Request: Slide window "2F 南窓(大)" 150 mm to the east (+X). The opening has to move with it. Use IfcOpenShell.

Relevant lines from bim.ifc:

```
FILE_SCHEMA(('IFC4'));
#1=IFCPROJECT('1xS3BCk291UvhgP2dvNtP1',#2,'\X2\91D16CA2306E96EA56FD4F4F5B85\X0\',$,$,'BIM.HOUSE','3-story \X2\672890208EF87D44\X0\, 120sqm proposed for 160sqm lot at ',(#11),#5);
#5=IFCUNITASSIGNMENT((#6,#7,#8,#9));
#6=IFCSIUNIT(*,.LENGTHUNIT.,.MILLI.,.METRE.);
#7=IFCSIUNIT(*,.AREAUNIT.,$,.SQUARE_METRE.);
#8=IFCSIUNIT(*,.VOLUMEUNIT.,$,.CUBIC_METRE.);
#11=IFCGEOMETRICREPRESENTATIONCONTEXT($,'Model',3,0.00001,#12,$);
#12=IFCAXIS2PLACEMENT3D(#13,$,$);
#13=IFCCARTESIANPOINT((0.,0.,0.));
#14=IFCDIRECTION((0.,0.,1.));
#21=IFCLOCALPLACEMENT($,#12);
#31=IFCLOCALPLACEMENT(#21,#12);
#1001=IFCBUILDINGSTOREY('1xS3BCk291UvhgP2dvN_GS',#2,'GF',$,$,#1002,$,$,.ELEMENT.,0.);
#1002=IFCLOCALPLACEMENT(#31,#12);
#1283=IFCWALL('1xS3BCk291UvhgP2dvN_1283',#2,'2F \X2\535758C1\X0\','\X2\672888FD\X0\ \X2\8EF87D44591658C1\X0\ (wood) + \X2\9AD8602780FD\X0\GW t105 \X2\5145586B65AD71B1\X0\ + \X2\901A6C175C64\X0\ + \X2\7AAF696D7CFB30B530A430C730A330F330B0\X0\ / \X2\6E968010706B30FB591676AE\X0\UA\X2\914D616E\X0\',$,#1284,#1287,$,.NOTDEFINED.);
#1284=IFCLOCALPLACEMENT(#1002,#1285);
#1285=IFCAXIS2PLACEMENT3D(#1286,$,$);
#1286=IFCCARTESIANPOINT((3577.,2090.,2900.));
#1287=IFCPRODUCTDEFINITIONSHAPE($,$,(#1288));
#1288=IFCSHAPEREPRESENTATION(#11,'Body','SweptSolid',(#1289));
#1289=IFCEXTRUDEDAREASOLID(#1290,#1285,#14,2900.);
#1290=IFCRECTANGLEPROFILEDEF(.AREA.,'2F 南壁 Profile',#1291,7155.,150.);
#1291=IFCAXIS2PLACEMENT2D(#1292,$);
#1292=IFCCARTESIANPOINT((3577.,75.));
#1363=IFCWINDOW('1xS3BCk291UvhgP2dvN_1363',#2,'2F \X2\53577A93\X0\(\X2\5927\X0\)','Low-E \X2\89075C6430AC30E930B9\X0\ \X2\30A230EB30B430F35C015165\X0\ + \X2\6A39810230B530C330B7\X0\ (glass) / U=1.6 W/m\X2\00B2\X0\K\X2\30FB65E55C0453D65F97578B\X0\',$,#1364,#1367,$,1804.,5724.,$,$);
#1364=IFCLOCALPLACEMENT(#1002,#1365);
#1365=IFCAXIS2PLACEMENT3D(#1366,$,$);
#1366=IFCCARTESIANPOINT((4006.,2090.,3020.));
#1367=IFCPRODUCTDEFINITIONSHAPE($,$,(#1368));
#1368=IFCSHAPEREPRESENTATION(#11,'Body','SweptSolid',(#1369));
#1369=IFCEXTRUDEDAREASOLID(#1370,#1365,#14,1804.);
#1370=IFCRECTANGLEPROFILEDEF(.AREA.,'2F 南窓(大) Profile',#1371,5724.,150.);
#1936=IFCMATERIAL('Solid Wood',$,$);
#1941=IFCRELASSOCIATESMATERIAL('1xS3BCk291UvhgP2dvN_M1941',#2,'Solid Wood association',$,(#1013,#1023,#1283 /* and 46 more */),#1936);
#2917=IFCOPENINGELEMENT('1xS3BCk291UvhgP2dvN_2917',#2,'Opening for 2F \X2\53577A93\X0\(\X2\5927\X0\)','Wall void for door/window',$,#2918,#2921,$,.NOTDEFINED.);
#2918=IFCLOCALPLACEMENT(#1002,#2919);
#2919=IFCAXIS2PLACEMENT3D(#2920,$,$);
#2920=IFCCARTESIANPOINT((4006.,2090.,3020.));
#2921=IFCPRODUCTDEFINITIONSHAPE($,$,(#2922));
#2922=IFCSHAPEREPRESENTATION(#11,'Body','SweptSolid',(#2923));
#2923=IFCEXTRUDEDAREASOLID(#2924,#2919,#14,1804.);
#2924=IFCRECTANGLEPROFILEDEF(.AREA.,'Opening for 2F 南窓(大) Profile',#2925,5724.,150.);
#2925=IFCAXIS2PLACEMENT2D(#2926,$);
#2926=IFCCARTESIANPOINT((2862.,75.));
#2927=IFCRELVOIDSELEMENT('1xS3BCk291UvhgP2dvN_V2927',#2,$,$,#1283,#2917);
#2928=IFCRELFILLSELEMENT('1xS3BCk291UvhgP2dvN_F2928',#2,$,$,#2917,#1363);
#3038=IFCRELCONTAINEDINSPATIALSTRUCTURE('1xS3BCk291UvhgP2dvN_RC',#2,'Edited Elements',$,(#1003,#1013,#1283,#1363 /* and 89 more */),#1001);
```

```python
import ifcopenshell
import ifcopenshell.api.geometry
import ifcopenshell.util.placement
import ifcopenshell.util.unit

model = ifcopenshell.open("bim.ifc")
unit_scale = ifcopenshell.util.unit.calculate_unit_scale(model)

window = model.by_guid("1xS3BCk291UvhgP2dvN_1363")
opening = window.FillsVoids[0].RelatingOpeningElement
wall = opening.VoidsElements[0].RelatingBuildingElement

wall_matrix = ifcopenshell.util.placement.get_local_placement(wall.ObjectPlacement)
shift = wall_matrix[:3, 0] * 0.15 / unit_scale
before = ifcopenshell.util.placement.get_local_placement(window.ObjectPlacement)[:3, 3].copy()

# The window is not placed relative to its opening, so move both.
for product in (opening, window):
    matrix = ifcopenshell.util.placement.get_local_placement(product.ObjectPlacement)
    matrix[:3, 3] += shift
    ifcopenshell.api.geometry.edit_object_placement(model, product=product, matrix=matrix, is_si=False)

after = ifcopenshell.util.placement.get_local_placement(window.ObjectPlacement)[:3, 3]
print("window moved by", (after - before).round(3) + 0.0)

model.write("bim_v2.ifc")
```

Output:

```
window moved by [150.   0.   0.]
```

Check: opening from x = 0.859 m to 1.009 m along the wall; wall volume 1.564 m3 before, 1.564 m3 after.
